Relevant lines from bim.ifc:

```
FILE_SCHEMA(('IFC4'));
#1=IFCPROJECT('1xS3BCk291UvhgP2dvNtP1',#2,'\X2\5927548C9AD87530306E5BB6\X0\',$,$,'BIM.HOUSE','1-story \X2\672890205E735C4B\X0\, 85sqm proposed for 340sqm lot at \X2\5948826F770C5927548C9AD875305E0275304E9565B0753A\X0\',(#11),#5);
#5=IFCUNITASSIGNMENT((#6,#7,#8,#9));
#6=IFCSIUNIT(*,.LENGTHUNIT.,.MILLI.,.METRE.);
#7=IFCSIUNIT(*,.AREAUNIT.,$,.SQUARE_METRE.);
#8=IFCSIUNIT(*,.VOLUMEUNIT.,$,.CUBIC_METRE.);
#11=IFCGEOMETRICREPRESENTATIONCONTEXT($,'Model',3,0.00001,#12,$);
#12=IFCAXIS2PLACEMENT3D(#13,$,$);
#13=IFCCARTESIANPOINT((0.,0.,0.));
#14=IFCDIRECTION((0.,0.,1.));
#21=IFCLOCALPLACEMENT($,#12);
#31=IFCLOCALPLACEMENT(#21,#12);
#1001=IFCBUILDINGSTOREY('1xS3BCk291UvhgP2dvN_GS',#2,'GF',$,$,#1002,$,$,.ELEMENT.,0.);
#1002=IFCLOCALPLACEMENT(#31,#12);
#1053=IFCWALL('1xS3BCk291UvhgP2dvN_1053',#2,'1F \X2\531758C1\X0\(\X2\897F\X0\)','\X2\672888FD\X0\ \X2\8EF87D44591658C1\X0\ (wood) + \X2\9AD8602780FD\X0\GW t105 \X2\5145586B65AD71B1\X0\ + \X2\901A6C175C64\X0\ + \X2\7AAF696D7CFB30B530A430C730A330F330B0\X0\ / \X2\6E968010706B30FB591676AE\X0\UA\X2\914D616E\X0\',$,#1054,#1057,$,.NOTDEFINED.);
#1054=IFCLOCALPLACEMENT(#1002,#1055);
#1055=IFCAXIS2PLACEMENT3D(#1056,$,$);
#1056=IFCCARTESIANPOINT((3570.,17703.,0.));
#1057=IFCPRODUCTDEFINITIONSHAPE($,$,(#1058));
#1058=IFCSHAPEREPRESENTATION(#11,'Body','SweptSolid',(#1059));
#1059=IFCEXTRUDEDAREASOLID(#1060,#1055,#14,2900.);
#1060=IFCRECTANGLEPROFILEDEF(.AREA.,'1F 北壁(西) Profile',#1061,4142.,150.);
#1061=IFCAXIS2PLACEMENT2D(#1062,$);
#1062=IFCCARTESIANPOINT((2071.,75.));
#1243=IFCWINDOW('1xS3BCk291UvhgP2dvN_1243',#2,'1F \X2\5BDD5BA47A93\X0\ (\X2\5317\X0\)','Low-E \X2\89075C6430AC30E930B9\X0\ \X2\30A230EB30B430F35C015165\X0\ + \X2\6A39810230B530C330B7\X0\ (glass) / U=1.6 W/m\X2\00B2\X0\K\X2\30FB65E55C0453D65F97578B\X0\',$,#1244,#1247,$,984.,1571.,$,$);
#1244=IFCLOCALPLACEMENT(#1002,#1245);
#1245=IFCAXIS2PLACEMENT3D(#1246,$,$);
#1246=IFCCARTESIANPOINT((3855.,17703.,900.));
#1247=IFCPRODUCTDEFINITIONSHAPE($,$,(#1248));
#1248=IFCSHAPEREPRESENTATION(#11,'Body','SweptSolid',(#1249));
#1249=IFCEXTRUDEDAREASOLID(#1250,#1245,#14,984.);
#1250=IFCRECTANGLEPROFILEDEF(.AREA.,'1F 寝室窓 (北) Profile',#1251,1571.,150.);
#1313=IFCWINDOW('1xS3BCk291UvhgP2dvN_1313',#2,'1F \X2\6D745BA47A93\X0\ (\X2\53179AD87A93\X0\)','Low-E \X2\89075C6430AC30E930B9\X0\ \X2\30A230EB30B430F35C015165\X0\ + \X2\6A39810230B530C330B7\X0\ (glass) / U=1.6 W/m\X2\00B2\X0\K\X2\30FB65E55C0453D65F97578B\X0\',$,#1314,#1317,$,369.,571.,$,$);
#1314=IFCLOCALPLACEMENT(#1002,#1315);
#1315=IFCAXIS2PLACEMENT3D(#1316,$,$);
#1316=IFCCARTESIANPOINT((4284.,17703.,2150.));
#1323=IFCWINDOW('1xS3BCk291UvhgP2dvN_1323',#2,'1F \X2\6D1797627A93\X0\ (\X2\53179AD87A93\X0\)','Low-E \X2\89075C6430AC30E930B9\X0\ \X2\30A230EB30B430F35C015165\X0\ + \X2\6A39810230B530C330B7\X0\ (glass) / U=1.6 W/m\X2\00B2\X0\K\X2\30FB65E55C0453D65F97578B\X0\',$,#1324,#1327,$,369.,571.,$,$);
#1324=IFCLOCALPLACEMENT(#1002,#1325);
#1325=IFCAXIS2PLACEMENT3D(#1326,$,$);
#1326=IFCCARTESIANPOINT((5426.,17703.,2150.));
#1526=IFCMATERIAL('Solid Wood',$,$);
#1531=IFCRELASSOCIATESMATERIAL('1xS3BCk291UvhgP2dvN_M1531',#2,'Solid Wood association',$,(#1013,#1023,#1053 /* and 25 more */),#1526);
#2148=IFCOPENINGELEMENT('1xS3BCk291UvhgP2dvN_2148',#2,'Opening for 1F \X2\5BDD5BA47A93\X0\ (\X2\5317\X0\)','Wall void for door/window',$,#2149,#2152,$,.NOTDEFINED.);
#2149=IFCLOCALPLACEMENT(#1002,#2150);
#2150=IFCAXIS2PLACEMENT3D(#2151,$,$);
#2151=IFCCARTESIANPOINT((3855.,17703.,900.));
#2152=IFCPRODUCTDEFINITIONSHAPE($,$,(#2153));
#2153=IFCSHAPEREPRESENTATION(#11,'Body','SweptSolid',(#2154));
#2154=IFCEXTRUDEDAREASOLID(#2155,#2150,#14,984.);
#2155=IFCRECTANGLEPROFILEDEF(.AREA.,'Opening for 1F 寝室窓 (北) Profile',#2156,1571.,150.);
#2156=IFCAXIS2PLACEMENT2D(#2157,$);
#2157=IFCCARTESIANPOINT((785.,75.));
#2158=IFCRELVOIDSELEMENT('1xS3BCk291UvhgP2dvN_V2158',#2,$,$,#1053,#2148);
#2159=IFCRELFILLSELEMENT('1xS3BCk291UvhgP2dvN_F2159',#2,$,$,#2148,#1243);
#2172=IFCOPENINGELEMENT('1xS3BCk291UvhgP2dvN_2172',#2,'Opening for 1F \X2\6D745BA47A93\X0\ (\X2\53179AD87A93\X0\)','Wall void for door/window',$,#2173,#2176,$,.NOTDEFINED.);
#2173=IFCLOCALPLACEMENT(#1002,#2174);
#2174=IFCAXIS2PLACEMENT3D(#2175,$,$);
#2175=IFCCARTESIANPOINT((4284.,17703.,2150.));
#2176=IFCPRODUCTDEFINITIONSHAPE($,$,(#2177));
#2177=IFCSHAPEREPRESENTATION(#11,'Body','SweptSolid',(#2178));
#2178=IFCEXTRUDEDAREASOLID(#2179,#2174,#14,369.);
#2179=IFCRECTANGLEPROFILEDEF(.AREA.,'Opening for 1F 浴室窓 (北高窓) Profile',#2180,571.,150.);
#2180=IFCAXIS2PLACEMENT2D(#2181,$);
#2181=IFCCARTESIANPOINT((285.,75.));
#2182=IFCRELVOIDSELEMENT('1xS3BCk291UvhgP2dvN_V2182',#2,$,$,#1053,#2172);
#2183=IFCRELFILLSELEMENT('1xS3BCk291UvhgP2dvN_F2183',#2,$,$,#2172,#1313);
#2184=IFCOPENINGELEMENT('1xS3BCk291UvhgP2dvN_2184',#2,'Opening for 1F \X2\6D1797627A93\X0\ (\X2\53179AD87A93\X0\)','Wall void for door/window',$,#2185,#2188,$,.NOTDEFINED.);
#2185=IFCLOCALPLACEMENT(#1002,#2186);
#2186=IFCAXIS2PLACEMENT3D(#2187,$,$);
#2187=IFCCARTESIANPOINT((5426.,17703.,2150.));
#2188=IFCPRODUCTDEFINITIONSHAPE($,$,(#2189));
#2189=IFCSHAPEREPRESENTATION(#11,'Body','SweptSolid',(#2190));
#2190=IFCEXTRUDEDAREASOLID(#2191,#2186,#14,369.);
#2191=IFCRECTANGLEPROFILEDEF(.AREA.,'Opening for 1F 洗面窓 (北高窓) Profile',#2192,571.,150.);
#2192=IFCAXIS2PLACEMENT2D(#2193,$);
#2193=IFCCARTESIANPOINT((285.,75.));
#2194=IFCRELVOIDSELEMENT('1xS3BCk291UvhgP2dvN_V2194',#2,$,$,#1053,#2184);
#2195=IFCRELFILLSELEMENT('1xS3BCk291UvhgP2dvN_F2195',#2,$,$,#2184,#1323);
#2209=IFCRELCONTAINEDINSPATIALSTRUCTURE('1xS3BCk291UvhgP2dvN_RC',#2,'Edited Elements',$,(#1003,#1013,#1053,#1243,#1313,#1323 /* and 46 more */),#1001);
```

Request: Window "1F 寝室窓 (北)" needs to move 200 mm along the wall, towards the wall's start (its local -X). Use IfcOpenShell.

```python
import ifcopenshell
import ifcopenshell.api.geometry
import ifcopenshell.util.placement
import ifcopenshell.util.unit

model = ifcopenshell.open("bim.ifc")
unit_scale = ifcopenshell.util.unit.calculate_unit_scale(model)

window = model.by_guid("1xS3BCk291UvhgP2dvN_1243")
opening = window.FillsVoids[0].RelatingOpeningElement
wall = opening.VoidsElements[0].RelatingBuildingElement

wall_matrix = ifcopenshell.util.placement.get_local_placement(wall.ObjectPlacement)
shift = wall_matrix[:3, 0] * -0.2 / unit_scale
before = ifcopenshell.util.placement.get_local_placement(window.ObjectPlacement)[:3, 3].copy()

# The window is not placed relative to its opening, so move both.
for product in (opening, window):
    matrix = ifcopenshell.util.placement.get_local_placement(product.ObjectPlacement)
    matrix[:3, 3] += shift
    ifcopenshell.api.geometry.edit_object_placement(model, product=product, matrix=matrix, is_si=False)

after = ifcopenshell.util.placement.get_local_placement(window.ObjectPlacement)[:3, 3]
print("window moved by", (after - before).round(3) + 0.0)

model.write("bim_edited.ifc")
```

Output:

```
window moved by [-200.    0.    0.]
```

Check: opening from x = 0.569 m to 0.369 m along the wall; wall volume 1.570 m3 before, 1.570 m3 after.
